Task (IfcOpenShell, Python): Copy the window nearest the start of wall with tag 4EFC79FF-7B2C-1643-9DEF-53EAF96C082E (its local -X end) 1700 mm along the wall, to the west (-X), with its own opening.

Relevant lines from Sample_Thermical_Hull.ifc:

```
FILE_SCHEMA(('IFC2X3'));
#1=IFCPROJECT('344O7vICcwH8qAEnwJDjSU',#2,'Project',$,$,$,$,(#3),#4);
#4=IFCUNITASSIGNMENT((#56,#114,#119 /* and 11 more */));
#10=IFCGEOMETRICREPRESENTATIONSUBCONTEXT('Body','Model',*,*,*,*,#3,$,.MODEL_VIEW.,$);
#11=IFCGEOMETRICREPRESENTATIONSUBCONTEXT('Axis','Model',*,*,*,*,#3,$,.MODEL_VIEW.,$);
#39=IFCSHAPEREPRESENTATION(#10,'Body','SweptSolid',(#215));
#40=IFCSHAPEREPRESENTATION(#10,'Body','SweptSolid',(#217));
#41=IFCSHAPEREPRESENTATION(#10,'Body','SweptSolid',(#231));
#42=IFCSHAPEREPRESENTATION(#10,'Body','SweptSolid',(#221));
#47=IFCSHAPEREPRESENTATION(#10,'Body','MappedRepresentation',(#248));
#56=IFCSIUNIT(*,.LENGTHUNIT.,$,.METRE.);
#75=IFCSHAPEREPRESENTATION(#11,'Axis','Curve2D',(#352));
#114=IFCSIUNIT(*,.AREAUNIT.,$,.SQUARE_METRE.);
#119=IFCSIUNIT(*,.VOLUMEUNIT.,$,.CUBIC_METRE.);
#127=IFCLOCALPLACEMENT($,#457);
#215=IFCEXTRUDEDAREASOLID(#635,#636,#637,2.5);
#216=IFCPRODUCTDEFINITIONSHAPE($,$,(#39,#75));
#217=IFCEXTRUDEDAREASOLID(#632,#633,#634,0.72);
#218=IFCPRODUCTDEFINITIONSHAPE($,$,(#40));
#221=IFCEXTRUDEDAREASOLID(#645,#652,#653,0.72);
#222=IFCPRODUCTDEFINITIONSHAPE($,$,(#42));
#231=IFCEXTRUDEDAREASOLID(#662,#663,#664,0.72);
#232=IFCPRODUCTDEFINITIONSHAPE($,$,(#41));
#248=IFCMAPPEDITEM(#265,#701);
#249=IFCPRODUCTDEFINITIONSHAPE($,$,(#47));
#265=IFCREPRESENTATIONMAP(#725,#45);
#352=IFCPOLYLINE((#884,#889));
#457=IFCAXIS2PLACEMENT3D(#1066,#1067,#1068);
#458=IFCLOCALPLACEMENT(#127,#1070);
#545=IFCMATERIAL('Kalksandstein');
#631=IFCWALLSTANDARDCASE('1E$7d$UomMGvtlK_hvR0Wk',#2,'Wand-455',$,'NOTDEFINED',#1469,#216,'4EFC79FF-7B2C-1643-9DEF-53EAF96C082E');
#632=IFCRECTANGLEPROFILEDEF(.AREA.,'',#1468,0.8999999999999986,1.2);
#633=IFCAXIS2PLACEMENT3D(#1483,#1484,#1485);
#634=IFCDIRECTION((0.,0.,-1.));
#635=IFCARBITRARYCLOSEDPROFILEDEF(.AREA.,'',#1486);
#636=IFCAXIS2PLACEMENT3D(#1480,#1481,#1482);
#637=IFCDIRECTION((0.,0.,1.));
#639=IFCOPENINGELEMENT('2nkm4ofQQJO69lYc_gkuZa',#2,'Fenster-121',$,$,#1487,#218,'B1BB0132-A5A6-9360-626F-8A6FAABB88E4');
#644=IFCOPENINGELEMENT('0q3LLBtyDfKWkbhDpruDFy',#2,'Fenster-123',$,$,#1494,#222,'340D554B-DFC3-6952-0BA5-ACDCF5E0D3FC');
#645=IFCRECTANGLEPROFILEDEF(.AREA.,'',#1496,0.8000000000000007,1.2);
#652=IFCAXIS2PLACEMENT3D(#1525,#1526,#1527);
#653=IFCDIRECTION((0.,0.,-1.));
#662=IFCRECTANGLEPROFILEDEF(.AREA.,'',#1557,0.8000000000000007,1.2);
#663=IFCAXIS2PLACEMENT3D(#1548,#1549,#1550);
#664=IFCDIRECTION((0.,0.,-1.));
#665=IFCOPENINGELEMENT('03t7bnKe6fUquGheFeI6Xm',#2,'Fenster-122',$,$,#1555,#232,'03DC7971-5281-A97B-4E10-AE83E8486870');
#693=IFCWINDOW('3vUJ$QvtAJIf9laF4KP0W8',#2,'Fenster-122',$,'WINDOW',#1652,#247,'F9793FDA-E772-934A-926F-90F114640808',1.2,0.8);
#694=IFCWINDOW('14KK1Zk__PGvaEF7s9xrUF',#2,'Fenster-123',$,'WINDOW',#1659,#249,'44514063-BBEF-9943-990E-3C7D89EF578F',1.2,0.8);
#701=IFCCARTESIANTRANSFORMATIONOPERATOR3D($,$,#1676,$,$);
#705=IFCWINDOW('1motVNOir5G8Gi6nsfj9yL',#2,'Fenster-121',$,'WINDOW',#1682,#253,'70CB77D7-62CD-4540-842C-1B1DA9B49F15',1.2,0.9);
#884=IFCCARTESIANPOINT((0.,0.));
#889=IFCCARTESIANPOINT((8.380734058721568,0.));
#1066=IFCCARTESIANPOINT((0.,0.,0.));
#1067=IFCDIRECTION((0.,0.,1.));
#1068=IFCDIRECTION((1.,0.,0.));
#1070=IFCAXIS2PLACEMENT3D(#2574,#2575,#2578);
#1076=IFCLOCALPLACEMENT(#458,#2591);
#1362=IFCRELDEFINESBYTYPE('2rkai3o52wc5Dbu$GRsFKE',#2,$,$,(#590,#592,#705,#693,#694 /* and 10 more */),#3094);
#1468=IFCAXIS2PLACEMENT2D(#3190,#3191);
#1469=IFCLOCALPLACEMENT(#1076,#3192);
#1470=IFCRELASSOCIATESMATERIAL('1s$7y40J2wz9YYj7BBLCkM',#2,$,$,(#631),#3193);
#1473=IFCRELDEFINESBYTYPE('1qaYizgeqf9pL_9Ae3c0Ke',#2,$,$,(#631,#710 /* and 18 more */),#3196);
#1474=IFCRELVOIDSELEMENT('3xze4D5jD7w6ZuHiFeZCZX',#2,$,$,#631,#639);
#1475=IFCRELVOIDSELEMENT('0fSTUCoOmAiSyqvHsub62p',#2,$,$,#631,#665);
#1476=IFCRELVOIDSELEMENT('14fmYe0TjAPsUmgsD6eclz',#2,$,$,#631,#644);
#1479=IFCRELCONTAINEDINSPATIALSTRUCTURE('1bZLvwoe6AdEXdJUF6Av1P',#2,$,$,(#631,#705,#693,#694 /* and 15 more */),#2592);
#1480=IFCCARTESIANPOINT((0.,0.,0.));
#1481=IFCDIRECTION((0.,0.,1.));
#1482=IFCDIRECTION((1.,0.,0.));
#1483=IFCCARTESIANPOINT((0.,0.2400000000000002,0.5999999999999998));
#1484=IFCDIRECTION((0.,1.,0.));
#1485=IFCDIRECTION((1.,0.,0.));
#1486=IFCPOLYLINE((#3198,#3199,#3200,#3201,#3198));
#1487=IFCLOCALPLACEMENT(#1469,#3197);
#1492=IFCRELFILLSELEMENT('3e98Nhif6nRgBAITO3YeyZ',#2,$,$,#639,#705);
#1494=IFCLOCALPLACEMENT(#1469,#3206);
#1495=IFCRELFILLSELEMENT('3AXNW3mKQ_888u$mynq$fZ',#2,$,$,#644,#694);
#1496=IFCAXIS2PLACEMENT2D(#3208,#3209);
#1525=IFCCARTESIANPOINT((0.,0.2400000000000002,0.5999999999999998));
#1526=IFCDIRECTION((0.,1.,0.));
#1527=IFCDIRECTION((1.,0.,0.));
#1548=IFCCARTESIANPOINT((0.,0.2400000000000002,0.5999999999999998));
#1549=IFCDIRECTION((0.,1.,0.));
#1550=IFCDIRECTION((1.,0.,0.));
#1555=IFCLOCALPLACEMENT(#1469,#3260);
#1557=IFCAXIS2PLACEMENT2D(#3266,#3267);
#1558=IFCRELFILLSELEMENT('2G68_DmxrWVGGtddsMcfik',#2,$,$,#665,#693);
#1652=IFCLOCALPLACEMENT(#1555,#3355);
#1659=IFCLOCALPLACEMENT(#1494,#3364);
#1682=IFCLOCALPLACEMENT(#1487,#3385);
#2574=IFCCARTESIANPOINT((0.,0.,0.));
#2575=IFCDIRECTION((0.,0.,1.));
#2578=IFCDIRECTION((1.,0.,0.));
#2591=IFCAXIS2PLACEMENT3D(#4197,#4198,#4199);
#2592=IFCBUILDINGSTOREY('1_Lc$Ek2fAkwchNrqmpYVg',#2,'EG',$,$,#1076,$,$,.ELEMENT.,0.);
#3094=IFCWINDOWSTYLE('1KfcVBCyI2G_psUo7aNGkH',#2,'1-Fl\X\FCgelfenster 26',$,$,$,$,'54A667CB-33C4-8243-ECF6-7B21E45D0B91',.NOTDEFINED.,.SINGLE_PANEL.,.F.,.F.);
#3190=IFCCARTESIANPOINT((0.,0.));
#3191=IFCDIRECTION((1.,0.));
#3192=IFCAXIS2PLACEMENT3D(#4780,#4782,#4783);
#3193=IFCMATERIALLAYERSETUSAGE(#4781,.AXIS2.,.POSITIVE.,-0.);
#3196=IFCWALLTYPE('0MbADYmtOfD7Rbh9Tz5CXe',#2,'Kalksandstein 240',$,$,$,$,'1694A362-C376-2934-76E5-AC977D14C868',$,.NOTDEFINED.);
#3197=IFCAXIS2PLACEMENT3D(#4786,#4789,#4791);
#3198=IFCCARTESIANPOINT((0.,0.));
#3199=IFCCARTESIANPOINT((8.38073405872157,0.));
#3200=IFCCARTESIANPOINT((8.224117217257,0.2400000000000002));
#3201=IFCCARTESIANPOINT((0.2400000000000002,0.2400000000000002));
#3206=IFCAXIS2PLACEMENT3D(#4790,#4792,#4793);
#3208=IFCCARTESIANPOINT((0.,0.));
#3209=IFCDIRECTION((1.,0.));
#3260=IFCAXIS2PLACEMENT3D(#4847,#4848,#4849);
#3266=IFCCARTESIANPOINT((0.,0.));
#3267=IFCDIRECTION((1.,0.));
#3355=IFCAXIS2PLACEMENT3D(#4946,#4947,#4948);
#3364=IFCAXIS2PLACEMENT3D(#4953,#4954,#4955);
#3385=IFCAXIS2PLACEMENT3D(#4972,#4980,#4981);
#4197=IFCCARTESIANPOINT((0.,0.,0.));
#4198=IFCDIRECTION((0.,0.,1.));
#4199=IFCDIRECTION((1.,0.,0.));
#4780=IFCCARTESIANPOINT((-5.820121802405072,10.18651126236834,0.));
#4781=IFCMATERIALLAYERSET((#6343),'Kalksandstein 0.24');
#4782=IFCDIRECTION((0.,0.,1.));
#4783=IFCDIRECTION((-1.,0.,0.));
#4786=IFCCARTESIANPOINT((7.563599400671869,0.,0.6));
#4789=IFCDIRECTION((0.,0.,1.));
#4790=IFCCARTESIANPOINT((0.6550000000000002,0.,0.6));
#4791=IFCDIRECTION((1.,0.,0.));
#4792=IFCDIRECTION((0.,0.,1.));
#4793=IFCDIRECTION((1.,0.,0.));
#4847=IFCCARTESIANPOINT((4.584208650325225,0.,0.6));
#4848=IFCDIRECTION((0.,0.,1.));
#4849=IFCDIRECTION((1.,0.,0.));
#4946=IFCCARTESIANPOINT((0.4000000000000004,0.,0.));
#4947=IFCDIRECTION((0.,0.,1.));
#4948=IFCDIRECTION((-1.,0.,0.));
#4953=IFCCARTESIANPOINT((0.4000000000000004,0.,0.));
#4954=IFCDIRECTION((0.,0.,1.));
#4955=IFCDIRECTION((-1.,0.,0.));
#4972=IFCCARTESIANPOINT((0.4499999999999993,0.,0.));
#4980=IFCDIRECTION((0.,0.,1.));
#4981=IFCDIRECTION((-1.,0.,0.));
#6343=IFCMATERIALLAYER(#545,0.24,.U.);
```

```python
import ifcopenshell
import ifcopenshell.api.feature
import ifcopenshell.api.geometry
import ifcopenshell.api.root
import ifcopenshell.geom
import ifcopenshell.util.element
import ifcopenshell.util.placement
import ifcopenshell.util.shape

model = ifcopenshell.open("Sample_Thermical_Hull.ifc")
settings = ifcopenshell.geom.settings()


def volume(element):
    """Net volume in cubic metres, openings subtracted."""
    shape = ifcopenshell.geom.create_shape(settings, element)
    return ifcopenshell.util.shape.get_volume(shape.geometry)


def reuse_history(source, copy):
    """copy_class also copies each property set's owner history, people and application; keep the originals."""
    for rel in copy.IsDefinedBy:
        if rel.is_a("IfcRelDefinesByProperties") and (history := rel.RelatingPropertyDefinition.OwnerHistory):
            rel.RelatingPropertyDefinition.OwnerHistory = source.OwnerHistory
            ifcopenshell.util.element.remove_deep2(model, history)


window = model.by_id(694)
opening = window.FillsVoids[0].RelatingOpeningElement
wall = opening.VoidsElements[0].RelatingBuildingElement
before = volume(wall)
shift = ifcopenshell.util.placement.get_local_placement(wall.ObjectPlacement)[:3, 0] * 1.7

# copy_class copies the void relationship, type, container and properties, but no geometry.
new_opening = ifcopenshell.api.root.copy_class(model, product=opening)
new_opening.Representation = ifcopenshell.util.element.copy_deep(
    model, opening.Representation, exclude=["IfcGeometricRepresentationContext", "IfcRepresentationMap"]
)
new_opening.Tag = None
new_window = ifcopenshell.api.root.copy_class(model, product=window)
new_window.Representation = ifcopenshell.util.element.copy_deep(
    model, window.Representation, exclude=["IfcGeometricRepresentationContext", "IfcRepresentationMap"]
)
new_window.Tag = None
reuse_history(window, new_window)
fills = ifcopenshell.api.feature.add_filling(model, opening=new_opening, element=new_window)
fills.OwnerHistory = new_window.OwnerHistory  # required in IFC2X3

for old, new in ((opening, new_opening), (window, new_window)):
    matrix = ifcopenshell.util.placement.get_local_placement(old.ObjectPlacement)
    matrix[:3, 3] += shift
    ifcopenshell.api.geometry.edit_object_placement(model, product=new, matrix=matrix, is_si=False)

after = volume(wall)

print(f"wall volume {before:.3f} -> {after:.3f} m3")

model.write("Sample_Thermical_Hull_rev.ifc")
```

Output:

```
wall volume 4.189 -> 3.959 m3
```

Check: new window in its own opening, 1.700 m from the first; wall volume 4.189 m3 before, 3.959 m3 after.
